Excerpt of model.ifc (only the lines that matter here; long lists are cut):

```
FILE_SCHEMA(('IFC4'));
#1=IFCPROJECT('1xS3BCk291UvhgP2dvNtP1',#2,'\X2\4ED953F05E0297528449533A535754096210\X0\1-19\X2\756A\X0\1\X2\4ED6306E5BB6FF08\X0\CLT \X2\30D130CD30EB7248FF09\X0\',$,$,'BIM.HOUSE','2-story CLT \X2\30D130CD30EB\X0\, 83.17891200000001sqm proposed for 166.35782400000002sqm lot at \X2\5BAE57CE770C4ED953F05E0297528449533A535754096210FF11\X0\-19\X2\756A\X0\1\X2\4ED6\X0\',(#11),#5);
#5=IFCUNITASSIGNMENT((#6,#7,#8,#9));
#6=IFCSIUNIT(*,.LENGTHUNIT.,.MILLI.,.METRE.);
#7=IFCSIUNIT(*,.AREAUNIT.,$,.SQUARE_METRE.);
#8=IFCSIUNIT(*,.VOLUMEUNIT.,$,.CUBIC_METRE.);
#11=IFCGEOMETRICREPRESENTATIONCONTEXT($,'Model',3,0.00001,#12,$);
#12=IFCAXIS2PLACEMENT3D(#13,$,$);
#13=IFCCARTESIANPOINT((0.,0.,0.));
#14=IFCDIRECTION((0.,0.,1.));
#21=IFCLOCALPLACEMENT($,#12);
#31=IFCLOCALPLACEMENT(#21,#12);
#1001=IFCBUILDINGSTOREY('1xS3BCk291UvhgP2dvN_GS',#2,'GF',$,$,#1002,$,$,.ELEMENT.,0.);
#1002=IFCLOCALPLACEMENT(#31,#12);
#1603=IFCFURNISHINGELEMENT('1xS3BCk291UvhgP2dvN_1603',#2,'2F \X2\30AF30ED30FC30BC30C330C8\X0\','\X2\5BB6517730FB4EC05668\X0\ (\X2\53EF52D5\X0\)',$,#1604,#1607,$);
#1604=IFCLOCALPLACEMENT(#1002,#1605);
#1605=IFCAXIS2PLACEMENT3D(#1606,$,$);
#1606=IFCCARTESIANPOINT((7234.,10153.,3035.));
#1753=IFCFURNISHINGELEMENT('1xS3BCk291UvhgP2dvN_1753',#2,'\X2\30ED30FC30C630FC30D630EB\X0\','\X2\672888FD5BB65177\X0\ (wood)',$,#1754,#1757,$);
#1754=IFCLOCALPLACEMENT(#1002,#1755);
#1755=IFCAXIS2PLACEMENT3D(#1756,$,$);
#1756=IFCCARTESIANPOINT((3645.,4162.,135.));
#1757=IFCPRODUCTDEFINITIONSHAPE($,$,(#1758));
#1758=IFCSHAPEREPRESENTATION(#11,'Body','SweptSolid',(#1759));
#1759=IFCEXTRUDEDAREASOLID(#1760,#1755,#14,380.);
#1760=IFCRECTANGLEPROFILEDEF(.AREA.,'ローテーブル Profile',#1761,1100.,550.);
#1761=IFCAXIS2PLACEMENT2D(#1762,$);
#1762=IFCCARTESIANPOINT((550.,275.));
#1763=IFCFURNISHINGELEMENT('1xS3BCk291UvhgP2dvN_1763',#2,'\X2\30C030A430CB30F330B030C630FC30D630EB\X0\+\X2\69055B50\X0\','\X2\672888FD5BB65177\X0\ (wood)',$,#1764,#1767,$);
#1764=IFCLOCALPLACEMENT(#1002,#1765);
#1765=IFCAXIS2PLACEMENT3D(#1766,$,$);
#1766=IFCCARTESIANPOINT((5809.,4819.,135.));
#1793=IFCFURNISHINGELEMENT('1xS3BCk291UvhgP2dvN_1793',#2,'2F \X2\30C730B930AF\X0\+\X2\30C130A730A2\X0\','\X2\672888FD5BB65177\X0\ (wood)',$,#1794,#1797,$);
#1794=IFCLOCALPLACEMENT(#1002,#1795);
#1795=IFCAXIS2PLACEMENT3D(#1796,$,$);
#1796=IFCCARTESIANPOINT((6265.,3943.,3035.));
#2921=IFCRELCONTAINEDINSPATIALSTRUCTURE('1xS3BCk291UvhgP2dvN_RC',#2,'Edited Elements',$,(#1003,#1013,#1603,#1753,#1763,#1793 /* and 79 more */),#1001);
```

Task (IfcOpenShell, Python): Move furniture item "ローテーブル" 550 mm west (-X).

```python
import ifcopenshell
import ifcopenshell.api.geometry
import ifcopenshell.util.placement
import ifcopenshell.util.unit

model = ifcopenshell.open("model.ifc")
unit_scale = ifcopenshell.util.unit.calculate_unit_scale(model)

item = model.by_guid("1xS3BCk291UvhgP2dvN_1753")
matrix = ifcopenshell.util.placement.get_local_placement(item.ObjectPlacement)
matrix[0, 3] -= 0.55 / unit_scale
ifcopenshell.api.geometry.edit_object_placement(model, product=item, matrix=matrix, is_si=False)

print(ifcopenshell.util.placement.get_local_placement(item.ObjectPlacement).round(3) + 0.0)

model.write("model-out.ifc")
```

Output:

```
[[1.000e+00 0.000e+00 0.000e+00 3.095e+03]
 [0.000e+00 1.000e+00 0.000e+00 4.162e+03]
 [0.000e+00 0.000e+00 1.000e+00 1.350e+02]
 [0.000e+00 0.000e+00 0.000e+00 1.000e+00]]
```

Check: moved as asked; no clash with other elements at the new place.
